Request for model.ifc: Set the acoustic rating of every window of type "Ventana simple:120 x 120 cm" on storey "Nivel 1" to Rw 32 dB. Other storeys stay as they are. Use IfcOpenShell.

First a look at what the model holds.

```python
import ifcopenshell
import ifcopenshell.util.element

model = ifcopenshell.open("model.ifc")
print(model.schema)
storey = next(s for s in model.by_type("IfcBuildingStorey") if s.Name == "Nivel 1")
windows = [e for e in ifcopenshell.util.element.get_decomposition(storey) if e.is_a("IfcWindow")]
seen = {}
for e in windows:
    element_type = ifcopenshell.util.element.get_type(e)
    key = (element_type.Name if element_type != e and element_type else None, ifcopenshell.util.element.get_pset(e, "Pset_WindowCommon", "AcousticRating"))
    seen[key] = seen.get(key, 0) + 1
for (name, value), count in sorted(seen.items(), key=str):
    print(count, "x", name, "|", value)
```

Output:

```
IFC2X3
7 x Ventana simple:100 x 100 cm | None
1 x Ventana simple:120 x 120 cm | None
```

```python
import ifcopenshell
import ifcopenshell.api.pset
import ifcopenshell.util.element

model = ifcopenshell.open("model.ifc")

storey = next(s for s in model.by_type("IfcBuildingStorey") if s.Name == "Nivel 1")
windows = [e for e in ifcopenshell.util.element.get_decomposition(storey) if e.is_a("IfcWindow")]

count = 0
for e in windows:
    element_type = ifcopenshell.util.element.get_type(e)
    if element_type in (None, e) or element_type.Name != "Ventana simple:120 x 120 cm":
        continue
    # add_pset returns the element's existing set when there is one.
    pset = ifcopenshell.api.pset.add_pset(model, product=e, name="Pset_WindowCommon")
    ifcopenshell.api.pset.edit_pset(model, pset=pset, properties={"AcousticRating": "Rw 32 dB"})
    count += 1

print(count, "windows updated")

model.write("model_rev.ifc")
```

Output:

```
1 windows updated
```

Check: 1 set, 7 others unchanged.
